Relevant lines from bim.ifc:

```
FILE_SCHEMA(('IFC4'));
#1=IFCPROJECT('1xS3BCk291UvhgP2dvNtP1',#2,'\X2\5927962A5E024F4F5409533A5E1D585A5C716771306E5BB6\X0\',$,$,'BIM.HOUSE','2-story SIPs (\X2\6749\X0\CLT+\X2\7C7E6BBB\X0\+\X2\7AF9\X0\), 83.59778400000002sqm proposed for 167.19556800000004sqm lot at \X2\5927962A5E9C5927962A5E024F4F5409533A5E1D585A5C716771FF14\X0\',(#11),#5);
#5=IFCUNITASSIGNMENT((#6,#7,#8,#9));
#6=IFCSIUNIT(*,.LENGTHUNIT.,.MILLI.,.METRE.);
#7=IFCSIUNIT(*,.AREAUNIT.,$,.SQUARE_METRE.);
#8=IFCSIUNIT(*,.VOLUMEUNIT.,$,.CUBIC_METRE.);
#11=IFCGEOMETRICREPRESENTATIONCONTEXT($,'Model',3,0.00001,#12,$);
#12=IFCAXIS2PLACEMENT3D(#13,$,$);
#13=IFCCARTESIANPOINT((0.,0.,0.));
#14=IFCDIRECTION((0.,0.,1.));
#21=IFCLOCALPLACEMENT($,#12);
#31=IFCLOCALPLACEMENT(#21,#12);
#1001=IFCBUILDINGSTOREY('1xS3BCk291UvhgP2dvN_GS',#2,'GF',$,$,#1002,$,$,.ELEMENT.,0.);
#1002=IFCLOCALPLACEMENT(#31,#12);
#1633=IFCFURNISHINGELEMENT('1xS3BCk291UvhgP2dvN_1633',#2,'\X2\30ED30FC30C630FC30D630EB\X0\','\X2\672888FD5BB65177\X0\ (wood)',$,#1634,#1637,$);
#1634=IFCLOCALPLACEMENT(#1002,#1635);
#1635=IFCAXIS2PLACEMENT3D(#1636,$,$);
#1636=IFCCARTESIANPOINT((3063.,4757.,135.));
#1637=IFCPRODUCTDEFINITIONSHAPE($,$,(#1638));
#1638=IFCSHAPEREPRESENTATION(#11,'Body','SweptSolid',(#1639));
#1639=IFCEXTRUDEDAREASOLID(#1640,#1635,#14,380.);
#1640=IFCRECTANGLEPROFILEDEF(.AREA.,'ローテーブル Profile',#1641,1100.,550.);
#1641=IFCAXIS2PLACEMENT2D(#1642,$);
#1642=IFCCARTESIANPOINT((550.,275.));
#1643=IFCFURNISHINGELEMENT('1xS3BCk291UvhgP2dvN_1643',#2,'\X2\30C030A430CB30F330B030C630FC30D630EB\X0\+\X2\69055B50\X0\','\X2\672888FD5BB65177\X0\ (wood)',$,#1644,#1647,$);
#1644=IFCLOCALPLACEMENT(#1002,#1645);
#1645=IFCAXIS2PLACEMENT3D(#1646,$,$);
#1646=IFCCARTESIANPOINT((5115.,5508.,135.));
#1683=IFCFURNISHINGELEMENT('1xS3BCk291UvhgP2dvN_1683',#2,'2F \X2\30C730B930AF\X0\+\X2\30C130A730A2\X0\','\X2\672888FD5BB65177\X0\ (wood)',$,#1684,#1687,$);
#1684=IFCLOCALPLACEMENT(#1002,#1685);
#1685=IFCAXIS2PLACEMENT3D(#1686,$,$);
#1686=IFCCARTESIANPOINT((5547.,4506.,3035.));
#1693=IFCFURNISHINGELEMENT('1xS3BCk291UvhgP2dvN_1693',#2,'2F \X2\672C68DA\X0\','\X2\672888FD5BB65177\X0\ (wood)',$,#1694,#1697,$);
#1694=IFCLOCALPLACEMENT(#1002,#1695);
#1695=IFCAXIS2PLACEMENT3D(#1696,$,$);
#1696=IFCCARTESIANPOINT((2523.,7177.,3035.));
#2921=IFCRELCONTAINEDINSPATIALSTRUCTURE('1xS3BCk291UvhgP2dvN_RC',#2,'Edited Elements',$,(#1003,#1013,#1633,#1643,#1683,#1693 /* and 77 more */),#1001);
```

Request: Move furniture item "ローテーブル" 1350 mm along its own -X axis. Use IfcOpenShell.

```python
import ifcopenshell
import ifcopenshell.api.geometry
import ifcopenshell.util.placement
import ifcopenshell.util.unit

model = ifcopenshell.open("bim.ifc")
unit_scale = ifcopenshell.util.unit.calculate_unit_scale(model)

item = model.by_guid("1xS3BCk291UvhgP2dvN_1633")
matrix = ifcopenshell.util.placement.get_local_placement(item.ObjectPlacement)
matrix[:3, 3] -= matrix[:3, 0] * 1.35 / unit_scale
ifcopenshell.api.geometry.edit_object_placement(model, product=item, matrix=matrix, is_si=False)

print(ifcopenshell.util.placement.get_local_placement(item.ObjectPlacement).round(3) + 0.0)

model.write("bim_rev.ifc")
```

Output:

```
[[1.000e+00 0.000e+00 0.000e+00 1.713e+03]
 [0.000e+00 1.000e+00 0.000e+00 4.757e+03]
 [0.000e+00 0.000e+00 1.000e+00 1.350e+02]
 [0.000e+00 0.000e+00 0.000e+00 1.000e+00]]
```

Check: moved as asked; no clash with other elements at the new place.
